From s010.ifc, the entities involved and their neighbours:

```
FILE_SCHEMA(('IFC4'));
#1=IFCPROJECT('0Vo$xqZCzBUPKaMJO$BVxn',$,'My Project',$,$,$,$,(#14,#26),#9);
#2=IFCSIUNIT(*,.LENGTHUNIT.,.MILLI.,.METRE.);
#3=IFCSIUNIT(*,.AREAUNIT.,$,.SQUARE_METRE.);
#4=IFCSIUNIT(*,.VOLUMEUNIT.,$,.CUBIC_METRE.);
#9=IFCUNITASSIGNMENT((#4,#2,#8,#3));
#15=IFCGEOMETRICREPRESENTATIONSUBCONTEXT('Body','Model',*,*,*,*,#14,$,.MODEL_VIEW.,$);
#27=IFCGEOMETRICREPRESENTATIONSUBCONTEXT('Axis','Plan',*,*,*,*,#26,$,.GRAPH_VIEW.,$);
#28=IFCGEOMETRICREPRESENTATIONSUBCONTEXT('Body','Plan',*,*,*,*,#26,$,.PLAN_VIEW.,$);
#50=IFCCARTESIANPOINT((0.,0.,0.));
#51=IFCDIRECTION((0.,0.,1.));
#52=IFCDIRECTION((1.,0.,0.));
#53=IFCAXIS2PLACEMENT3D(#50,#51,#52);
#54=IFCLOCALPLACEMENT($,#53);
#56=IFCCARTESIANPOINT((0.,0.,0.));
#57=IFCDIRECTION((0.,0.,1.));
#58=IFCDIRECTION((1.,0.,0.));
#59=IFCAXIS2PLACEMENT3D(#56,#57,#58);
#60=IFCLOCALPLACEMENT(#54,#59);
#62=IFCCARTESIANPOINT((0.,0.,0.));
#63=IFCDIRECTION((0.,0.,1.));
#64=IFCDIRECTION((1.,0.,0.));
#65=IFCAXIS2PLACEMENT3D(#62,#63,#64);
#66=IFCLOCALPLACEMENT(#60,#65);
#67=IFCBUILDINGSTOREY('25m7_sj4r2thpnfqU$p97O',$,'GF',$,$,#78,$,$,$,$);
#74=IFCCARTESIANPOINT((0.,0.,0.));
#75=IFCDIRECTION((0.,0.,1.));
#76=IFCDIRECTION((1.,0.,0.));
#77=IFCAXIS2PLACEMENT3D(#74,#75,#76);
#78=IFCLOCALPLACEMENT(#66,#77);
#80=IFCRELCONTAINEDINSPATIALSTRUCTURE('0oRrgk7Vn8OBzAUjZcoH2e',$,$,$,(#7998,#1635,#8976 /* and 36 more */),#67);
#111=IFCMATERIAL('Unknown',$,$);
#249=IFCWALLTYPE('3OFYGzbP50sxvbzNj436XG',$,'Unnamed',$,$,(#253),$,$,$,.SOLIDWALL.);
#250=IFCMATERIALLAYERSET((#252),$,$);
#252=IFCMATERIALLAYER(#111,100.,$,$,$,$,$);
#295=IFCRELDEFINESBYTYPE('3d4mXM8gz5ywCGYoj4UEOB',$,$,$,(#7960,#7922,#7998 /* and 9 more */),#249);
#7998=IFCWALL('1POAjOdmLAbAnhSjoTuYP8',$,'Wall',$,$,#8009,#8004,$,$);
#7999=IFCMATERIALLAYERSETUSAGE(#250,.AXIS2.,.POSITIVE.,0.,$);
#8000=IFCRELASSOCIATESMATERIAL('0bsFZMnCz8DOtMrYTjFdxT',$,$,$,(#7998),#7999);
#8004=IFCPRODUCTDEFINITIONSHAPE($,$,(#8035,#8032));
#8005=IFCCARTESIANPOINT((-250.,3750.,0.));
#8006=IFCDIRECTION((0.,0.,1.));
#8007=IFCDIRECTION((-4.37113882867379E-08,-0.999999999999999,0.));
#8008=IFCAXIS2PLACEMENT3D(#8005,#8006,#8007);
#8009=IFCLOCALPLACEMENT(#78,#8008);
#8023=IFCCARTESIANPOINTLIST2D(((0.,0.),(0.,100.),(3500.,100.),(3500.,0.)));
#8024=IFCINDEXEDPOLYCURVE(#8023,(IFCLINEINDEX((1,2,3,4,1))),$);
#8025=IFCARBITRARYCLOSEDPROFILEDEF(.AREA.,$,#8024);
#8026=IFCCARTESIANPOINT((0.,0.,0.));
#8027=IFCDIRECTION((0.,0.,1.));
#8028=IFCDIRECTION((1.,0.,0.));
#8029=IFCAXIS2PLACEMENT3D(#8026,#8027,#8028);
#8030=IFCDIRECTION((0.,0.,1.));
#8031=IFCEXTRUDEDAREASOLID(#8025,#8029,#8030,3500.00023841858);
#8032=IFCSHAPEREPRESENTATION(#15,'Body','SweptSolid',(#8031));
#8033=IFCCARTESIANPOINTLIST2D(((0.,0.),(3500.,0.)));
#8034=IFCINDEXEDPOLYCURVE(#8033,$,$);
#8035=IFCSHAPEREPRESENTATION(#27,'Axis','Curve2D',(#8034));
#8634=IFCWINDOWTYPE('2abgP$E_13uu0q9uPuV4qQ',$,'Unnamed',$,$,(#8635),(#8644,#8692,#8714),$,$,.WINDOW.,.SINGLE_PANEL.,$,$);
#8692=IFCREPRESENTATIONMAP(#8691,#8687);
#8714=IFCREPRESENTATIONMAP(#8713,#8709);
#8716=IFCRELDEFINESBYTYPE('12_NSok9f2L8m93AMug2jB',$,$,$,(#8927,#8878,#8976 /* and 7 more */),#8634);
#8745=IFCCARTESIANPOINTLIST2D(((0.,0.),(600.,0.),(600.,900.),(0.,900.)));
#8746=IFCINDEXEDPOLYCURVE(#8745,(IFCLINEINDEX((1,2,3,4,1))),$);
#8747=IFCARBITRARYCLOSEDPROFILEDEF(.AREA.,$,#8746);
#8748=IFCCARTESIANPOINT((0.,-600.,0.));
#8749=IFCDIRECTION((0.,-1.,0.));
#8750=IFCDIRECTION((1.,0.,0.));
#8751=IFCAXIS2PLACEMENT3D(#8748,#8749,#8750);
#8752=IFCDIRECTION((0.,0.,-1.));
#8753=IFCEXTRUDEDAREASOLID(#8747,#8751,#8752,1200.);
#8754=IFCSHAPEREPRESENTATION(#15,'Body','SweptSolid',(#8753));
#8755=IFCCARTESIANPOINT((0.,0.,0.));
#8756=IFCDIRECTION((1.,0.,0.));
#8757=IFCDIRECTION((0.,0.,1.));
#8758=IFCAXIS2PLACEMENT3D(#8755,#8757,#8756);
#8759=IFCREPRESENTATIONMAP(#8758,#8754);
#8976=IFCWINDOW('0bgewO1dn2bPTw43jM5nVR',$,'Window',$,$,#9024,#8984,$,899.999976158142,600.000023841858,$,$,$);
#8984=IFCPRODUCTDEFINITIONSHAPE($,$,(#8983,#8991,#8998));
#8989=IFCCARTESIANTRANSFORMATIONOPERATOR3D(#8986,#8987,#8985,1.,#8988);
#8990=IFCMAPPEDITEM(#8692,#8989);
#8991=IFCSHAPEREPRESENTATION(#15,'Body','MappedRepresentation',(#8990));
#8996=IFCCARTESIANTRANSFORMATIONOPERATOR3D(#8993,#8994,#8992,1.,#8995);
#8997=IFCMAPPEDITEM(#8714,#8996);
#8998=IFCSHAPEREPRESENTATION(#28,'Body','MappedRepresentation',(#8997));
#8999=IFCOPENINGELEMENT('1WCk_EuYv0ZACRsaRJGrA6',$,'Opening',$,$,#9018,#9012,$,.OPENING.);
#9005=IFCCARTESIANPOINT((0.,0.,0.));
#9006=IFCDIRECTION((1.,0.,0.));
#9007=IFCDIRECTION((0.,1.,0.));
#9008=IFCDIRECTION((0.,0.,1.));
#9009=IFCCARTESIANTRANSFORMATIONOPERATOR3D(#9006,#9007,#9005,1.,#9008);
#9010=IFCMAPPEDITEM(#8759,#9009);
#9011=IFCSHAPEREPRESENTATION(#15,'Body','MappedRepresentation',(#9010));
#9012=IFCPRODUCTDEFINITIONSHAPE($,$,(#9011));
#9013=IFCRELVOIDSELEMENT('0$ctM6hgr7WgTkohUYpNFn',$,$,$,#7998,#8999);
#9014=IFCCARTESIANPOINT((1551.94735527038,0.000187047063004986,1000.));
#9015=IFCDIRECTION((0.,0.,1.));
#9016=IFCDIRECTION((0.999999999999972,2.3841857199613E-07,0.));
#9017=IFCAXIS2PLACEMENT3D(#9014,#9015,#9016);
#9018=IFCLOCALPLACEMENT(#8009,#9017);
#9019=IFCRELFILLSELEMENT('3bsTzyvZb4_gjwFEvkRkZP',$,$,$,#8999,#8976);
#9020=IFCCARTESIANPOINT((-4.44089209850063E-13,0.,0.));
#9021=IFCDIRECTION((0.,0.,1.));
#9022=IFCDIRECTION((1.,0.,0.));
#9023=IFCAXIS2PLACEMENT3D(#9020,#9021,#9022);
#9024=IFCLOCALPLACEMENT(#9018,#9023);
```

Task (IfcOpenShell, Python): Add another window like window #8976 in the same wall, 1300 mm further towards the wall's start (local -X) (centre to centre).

```python
import ifcopenshell
import ifcopenshell.api.feature
import ifcopenshell.api.geometry
import ifcopenshell.api.root
import ifcopenshell.geom
import ifcopenshell.util.element
import ifcopenshell.util.placement
import ifcopenshell.util.shape
import ifcopenshell.util.unit

model = ifcopenshell.open("s010.ifc")
unit_scale = ifcopenshell.util.unit.calculate_unit_scale(model)
settings = ifcopenshell.geom.settings()


def volume(element):
    """Net volume in cubic metres, openings subtracted."""
    shape = ifcopenshell.geom.create_shape(settings, element)
    return ifcopenshell.util.shape.get_volume(shape.geometry)


window = model.by_guid("0bgewO1dn2bPTw43jM5nVR")
opening = window.FillsVoids[0].RelatingOpeningElement
wall = opening.VoidsElements[0].RelatingBuildingElement
before = volume(wall)
shift = ifcopenshell.util.placement.get_local_placement(wall.ObjectPlacement)[:3, 0] * -1.3 / unit_scale

# copy_class copies the void relationship, type, container and properties, but no geometry.
new_opening = ifcopenshell.api.root.copy_class(model, product=opening)
new_opening.Representation = ifcopenshell.util.element.copy_deep(
    model, opening.Representation, exclude=["IfcGeometricRepresentationContext", "IfcRepresentationMap"]
)
new_window = ifcopenshell.api.root.copy_class(model, product=window)
new_window.Representation = ifcopenshell.util.element.copy_deep(
    model, window.Representation, exclude=["IfcGeometricRepresentationContext", "IfcRepresentationMap"]
)
ifcopenshell.api.feature.add_filling(model, opening=new_opening, element=new_window)

for old, new in ((opening, new_opening), (window, new_window)):
    matrix = ifcopenshell.util.placement.get_local_placement(old.ObjectPlacement)
    matrix[:3, 3] += shift
    ifcopenshell.api.geometry.edit_object_placement(model, product=new, matrix=matrix, is_si=False)

after = volume(wall)

print(f"wall volume {before:.3f} -> {after:.3f} m3")

model.write("s010_v2.ifc")
```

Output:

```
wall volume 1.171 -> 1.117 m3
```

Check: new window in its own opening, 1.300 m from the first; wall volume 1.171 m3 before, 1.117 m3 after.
